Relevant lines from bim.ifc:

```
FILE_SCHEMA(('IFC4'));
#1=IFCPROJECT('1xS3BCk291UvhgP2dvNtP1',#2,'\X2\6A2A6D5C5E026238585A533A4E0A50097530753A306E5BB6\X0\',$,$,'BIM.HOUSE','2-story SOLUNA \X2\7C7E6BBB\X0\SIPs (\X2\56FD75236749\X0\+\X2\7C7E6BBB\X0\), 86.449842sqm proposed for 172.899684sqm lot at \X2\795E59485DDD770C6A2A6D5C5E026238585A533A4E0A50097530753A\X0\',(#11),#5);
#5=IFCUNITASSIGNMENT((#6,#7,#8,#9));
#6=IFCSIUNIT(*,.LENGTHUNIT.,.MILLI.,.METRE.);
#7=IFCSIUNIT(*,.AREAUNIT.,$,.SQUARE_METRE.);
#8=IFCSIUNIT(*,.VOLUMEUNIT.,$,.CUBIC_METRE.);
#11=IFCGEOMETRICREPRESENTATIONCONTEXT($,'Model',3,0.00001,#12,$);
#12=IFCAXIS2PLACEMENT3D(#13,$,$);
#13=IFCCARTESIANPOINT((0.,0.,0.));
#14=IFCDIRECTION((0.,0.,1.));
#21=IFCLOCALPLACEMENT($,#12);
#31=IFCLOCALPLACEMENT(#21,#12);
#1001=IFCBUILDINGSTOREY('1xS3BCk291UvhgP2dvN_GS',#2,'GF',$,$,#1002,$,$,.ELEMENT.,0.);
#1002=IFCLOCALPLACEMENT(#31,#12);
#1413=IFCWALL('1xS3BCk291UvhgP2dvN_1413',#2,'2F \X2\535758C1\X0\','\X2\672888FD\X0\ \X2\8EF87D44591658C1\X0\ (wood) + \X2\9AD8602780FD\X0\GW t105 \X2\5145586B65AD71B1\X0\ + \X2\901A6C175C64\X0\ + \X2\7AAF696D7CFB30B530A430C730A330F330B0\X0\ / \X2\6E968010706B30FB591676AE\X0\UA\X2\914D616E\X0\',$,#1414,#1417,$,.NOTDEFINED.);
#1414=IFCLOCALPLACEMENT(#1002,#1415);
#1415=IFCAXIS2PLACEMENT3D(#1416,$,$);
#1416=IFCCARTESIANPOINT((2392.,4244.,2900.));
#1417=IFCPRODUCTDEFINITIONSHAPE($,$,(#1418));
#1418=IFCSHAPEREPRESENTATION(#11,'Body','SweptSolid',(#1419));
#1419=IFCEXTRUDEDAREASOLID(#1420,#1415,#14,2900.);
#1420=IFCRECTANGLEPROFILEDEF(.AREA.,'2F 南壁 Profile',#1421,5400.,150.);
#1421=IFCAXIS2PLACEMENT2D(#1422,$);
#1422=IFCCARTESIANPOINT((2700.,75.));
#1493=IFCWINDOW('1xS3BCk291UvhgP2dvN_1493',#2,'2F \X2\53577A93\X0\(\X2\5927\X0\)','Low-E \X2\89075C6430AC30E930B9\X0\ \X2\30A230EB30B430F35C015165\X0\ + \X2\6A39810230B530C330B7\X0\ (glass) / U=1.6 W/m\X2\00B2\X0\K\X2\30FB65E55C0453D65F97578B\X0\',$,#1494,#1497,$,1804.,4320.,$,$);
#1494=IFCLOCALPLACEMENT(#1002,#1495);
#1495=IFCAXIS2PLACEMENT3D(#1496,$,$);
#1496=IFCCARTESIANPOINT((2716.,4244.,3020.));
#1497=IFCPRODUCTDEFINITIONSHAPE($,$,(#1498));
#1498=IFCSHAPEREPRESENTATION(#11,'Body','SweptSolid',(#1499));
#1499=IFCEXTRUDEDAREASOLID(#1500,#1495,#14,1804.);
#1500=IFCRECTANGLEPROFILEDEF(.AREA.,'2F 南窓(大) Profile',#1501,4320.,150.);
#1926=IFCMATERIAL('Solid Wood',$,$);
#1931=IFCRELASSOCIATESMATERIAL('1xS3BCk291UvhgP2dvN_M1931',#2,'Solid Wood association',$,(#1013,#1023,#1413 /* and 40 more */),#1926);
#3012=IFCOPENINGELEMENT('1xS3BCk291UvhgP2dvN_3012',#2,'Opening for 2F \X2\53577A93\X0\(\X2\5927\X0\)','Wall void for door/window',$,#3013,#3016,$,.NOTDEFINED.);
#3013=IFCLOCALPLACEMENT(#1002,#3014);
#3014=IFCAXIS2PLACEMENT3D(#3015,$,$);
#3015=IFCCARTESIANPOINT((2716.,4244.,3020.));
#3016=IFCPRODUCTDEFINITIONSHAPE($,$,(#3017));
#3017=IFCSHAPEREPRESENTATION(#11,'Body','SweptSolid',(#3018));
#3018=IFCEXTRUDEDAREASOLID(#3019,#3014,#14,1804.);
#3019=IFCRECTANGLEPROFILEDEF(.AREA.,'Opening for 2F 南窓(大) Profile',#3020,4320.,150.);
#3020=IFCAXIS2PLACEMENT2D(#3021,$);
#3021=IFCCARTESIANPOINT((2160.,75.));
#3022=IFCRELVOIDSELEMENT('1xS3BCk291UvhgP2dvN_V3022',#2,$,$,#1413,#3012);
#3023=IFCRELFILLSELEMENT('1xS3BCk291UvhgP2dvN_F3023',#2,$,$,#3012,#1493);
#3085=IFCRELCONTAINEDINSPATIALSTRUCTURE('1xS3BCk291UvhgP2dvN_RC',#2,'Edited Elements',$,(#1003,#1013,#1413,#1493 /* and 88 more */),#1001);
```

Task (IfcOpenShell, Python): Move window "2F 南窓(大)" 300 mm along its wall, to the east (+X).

```python
import ifcopenshell
import ifcopenshell.api.geometry
import ifcopenshell.util.placement

model = ifcopenshell.open("bim.ifc")

window = model.by_guid("1xS3BCk291UvhgP2dvN_1493")
opening = window.FillsVoids[0].RelatingOpeningElement
wall = opening.VoidsElements[0].RelatingBuildingElement

wall_matrix = ifcopenshell.util.placement.get_local_placement(wall.ObjectPlacement)
shift = wall_matrix[:3, 0] * 300.0
before = ifcopenshell.util.placement.get_local_placement(window.ObjectPlacement)[:3, 3].copy()

# The window is not placed relative to its opening, so move both.
for product in (opening, window):
    matrix = ifcopenshell.util.placement.get_local_placement(product.ObjectPlacement)
    matrix[:3, 3] += shift
    ifcopenshell.api.geometry.edit_object_placement(model, product=product, matrix=matrix, is_si=False)

after = ifcopenshell.util.placement.get_local_placement(window.ObjectPlacement)[:3, 3]
print("window moved by", (after - before).round(3) + 0.0)

model.write("bim_updated.ifc")
```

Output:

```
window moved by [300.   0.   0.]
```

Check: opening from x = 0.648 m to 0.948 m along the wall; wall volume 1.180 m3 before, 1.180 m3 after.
